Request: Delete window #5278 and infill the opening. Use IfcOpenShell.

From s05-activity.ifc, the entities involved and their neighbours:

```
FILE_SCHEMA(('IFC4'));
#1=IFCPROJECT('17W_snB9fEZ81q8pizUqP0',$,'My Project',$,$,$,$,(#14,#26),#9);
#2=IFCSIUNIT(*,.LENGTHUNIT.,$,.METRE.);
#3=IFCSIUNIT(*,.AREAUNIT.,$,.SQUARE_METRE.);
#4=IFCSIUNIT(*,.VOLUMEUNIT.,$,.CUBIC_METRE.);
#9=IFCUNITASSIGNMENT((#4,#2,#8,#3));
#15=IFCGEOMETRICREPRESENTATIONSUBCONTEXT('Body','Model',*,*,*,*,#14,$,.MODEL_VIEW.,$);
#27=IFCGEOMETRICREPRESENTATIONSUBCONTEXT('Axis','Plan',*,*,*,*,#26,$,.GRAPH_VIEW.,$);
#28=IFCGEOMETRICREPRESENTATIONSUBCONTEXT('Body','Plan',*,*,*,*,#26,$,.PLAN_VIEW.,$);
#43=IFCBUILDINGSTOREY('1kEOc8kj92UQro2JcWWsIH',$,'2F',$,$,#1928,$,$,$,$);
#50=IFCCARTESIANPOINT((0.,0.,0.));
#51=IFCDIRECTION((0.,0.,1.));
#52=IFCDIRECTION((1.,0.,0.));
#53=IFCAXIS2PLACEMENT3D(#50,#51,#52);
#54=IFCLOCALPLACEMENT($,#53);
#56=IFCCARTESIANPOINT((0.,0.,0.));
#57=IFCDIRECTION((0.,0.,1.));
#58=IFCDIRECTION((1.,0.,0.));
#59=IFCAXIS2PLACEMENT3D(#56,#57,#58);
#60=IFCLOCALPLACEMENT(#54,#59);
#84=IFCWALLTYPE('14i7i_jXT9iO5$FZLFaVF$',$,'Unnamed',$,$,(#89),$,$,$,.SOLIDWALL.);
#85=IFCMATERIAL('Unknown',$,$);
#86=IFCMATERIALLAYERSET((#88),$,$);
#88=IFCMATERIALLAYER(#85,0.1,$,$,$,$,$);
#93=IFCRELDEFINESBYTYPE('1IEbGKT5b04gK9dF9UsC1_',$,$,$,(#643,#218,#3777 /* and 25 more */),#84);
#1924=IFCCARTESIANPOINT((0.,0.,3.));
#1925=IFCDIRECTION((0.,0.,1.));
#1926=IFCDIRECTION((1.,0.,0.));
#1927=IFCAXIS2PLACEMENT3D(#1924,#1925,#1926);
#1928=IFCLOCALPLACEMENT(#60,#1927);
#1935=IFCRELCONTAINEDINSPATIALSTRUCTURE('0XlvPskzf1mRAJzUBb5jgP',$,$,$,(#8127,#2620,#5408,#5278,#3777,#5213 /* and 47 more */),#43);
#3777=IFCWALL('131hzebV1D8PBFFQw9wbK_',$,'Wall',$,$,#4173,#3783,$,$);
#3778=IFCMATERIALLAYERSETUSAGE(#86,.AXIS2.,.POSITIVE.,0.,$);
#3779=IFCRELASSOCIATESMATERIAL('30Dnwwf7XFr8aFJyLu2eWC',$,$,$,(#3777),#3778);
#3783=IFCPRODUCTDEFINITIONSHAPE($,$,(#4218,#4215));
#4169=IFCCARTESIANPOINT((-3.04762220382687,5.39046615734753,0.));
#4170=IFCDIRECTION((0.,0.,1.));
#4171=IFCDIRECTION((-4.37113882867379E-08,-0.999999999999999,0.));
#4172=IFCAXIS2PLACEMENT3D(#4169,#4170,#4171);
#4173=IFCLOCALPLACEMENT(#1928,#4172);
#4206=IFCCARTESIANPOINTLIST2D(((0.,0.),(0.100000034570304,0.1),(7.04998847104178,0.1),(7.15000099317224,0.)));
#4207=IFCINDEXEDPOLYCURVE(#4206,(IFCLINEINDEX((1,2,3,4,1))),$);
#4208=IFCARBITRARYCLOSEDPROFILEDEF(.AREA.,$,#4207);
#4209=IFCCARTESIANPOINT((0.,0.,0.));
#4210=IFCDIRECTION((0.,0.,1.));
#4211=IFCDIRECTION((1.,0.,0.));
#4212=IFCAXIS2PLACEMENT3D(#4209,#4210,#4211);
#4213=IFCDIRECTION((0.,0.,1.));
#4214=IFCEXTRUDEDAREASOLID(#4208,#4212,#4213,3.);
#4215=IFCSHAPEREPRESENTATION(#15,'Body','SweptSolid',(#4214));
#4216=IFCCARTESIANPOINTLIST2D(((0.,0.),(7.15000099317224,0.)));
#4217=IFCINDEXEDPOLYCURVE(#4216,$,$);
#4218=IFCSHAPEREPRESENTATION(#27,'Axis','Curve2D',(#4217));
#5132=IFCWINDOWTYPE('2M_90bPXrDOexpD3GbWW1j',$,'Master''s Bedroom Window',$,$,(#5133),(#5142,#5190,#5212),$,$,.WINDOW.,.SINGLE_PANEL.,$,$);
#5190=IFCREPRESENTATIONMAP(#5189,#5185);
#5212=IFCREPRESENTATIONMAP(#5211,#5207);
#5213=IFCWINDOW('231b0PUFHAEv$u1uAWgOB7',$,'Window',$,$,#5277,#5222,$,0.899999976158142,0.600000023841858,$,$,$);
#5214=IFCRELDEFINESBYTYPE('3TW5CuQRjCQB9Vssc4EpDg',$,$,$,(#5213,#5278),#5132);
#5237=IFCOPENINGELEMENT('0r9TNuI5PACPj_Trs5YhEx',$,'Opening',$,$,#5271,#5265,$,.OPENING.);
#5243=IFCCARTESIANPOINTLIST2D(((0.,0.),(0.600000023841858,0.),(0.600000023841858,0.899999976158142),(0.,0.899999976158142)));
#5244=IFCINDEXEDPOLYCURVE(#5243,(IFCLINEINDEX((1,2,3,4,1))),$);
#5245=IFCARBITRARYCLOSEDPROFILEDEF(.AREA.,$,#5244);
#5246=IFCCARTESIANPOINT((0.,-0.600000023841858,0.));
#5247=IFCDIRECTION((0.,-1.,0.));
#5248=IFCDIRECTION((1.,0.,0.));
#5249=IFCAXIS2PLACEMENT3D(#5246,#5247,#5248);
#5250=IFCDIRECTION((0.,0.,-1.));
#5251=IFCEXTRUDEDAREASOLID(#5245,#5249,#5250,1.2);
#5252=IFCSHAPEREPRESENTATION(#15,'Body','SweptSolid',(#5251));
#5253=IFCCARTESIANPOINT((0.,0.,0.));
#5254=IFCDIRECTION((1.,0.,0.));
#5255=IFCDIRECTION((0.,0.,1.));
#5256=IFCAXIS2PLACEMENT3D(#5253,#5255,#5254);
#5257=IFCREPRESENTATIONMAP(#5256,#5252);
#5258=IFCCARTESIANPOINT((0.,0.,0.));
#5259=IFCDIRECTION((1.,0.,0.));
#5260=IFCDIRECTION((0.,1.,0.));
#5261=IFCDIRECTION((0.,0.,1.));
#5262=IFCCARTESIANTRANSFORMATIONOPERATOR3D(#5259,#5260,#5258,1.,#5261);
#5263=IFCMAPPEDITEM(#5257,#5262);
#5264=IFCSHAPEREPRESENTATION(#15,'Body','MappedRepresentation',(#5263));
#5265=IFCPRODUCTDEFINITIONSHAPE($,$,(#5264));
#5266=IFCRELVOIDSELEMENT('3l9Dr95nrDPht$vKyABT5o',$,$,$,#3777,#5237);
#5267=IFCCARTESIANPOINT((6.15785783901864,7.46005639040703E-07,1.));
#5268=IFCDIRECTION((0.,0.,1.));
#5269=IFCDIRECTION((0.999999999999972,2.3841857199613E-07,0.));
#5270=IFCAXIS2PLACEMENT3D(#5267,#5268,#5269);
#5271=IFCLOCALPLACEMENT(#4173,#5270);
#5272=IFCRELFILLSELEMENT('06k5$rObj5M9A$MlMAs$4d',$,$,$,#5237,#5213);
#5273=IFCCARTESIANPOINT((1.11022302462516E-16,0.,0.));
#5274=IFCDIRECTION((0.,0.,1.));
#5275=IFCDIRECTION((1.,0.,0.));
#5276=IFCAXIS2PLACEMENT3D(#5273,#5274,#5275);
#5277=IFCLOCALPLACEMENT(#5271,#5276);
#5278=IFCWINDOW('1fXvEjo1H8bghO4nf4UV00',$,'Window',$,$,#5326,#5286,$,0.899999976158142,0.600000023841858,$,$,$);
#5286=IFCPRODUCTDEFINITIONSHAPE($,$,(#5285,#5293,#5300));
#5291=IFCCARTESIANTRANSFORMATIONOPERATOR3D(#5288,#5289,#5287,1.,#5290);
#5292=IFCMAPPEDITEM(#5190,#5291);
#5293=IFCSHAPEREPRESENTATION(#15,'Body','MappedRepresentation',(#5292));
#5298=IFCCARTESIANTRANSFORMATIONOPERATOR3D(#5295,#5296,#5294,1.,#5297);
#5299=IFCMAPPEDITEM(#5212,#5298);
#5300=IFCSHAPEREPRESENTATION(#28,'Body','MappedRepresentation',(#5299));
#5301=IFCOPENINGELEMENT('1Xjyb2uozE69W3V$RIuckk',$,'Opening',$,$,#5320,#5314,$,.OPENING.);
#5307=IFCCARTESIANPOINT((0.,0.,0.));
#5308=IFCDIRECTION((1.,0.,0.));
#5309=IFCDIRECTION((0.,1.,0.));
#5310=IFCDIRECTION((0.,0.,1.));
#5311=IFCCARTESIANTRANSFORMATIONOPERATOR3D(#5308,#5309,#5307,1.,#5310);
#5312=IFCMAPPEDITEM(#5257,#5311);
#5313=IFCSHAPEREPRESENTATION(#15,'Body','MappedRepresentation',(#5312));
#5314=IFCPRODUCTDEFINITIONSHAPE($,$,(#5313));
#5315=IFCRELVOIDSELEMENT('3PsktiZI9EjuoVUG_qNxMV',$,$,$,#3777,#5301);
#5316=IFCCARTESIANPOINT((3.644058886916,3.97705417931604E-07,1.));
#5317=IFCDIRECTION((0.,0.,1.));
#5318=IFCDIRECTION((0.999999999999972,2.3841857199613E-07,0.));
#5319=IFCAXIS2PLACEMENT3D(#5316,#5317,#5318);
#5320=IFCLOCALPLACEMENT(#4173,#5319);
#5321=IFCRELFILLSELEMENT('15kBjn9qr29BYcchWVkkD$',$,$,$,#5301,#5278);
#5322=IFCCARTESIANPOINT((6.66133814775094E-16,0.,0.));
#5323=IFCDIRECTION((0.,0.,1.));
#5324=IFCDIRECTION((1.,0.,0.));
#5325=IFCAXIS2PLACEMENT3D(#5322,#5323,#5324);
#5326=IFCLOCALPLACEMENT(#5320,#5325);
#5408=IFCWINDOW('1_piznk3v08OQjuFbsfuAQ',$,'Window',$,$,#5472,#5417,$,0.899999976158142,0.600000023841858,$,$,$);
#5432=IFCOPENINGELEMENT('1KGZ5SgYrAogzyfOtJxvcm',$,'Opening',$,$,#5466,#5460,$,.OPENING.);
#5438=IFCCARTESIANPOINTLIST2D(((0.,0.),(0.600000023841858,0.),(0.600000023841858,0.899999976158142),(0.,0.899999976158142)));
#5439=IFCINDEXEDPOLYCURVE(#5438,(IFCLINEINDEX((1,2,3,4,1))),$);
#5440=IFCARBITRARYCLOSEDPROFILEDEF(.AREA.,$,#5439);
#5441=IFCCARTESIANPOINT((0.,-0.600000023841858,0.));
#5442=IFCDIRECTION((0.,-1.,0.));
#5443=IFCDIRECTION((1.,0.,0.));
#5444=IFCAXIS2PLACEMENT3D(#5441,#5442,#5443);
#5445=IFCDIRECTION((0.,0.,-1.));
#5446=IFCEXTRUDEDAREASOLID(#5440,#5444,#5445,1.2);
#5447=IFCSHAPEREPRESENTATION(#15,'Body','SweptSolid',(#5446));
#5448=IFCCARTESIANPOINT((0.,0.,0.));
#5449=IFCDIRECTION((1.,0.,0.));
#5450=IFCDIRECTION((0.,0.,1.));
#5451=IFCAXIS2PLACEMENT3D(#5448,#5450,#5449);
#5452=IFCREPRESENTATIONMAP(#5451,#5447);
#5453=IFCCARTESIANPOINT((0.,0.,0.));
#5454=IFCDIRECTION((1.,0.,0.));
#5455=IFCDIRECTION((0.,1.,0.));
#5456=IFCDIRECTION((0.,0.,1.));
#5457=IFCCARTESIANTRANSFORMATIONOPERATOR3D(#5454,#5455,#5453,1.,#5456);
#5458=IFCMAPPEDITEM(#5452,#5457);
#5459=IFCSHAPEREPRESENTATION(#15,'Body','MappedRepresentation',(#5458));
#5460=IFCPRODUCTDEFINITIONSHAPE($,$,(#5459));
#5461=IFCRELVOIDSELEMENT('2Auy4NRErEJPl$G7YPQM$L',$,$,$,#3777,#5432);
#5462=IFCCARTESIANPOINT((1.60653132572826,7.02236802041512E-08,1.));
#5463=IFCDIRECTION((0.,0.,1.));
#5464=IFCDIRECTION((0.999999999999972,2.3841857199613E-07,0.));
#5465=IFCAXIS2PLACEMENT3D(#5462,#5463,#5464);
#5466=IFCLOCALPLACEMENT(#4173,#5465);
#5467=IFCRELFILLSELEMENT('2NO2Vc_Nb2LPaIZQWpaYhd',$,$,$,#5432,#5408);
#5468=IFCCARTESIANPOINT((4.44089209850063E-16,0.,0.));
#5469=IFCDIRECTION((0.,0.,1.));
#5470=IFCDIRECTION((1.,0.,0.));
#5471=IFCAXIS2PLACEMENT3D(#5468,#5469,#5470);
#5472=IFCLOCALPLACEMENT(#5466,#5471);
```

```python
import ifcopenshell
import ifcopenshell.api.feature
import ifcopenshell.api.root
import ifcopenshell.geom
import ifcopenshell.util.shape

model = ifcopenshell.open("s05-activity.ifc")
settings = ifcopenshell.geom.settings()


def volume(element):
    """Net volume in cubic metres, openings subtracted."""
    shape = ifcopenshell.geom.create_shape(settings, element)
    return ifcopenshell.util.shape.get_volume(shape.geometry)


window = model.by_guid("1fXvEjo1H8bghO4nf4UV00")
opening = window.FillsVoids[0].RelatingOpeningElement
wall = opening.VoidsElements[0].RelatingBuildingElement
before = volume(wall)

ifcopenshell.api.root.remove_product(model, product=window)
ifcopenshell.api.feature.remove_feature(model, feature=opening)

after = volume(wall)

print(f"wall volume {before:.3f} -> {after:.3f} m3")

model.write("s05-activity_v2.ifc")
```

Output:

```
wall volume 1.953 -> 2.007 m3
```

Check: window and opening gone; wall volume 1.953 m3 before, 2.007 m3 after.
